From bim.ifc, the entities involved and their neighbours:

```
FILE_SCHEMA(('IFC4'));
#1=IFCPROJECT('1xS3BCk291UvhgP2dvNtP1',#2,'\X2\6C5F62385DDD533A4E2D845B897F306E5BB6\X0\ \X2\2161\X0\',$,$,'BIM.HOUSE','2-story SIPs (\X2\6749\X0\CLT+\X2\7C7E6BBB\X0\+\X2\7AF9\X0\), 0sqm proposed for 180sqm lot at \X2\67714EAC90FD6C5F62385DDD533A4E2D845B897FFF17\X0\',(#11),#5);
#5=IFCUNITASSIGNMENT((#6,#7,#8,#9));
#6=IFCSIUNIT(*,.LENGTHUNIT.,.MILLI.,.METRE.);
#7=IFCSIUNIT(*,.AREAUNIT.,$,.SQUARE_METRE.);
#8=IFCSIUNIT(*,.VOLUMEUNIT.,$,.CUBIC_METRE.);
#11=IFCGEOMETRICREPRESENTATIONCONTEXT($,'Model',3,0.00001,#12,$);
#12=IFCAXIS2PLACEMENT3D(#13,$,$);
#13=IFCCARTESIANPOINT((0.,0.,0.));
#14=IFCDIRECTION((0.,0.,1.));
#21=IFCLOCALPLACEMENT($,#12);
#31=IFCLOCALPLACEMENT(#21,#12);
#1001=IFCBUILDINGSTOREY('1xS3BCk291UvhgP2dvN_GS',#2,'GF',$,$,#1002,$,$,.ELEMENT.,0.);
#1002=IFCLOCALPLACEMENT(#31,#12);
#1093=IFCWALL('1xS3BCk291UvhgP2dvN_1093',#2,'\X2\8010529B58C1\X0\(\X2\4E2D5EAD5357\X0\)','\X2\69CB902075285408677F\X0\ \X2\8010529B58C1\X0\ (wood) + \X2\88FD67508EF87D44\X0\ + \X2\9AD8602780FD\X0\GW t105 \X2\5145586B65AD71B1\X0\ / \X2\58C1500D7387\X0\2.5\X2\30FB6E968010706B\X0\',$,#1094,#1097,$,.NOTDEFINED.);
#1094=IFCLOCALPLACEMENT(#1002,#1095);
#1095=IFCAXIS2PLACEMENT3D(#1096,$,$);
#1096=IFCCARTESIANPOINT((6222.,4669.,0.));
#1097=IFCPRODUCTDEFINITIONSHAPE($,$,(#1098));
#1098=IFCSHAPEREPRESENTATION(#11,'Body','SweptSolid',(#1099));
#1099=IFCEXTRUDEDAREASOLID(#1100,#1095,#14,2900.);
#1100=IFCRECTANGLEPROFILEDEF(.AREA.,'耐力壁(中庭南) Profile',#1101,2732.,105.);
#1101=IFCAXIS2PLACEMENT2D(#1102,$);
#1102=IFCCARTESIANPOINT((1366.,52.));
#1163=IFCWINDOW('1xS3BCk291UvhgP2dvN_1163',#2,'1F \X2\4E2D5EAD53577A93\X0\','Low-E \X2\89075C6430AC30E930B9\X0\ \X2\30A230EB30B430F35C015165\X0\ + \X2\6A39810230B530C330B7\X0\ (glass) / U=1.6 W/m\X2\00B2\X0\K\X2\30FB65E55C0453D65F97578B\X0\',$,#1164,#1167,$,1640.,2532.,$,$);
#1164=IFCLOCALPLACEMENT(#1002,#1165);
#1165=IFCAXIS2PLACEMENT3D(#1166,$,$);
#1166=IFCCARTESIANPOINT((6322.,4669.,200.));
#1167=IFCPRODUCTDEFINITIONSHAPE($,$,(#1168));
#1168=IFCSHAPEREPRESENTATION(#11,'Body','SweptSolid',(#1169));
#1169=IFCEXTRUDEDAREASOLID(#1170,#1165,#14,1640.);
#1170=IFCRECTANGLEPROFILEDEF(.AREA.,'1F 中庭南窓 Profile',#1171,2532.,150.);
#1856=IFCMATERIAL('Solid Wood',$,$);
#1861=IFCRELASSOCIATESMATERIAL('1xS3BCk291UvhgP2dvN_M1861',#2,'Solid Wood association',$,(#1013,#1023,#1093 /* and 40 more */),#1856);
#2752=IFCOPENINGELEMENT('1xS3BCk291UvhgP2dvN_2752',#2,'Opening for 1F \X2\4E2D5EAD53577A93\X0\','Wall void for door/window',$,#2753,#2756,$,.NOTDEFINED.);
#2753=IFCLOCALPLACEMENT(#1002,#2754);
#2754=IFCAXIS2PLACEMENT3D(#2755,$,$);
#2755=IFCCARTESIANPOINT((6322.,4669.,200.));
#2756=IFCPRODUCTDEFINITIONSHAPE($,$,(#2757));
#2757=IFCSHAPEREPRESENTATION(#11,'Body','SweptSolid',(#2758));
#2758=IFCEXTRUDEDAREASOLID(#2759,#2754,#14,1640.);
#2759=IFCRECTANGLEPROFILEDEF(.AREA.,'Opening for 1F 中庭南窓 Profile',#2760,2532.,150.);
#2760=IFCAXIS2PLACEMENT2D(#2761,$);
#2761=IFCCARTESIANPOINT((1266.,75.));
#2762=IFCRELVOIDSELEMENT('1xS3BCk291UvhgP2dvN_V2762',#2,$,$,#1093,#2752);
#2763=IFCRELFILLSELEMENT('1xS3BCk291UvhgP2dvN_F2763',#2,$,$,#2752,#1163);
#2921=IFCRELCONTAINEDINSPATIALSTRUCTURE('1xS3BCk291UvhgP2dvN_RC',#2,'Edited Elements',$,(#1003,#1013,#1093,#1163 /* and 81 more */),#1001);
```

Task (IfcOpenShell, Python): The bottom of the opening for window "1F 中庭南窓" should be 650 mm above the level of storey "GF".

```python
import numpy as np
import ifcopenshell
import ifcopenshell.api.geometry
import ifcopenshell.geom
import ifcopenshell.util.element
import ifcopenshell.util.placement
import ifcopenshell.util.shape
import ifcopenshell.util.unit

model = ifcopenshell.open("bim.ifc")
unit_scale = ifcopenshell.util.unit.calculate_unit_scale(model)

window = model.by_guid("1xS3BCk291UvhgP2dvN_1163")
opening = window.FillsVoids[0].RelatingOpeningElement
storey = ifcopenshell.util.element.get_container(window, ifc_class="IfcBuildingStorey")
level = ifcopenshell.util.placement.get_local_placement(storey.ObjectPlacement)[2, 3]

# The opening's origin need not be at the sill, so measure its lowest point.
shape = ifcopenshell.geom.create_shape(ifcopenshell.geom.settings(), opening)
bottom = ifcopenshell.util.shape.get_shape_bottom_elevation(shape, shape.geometry) / unit_scale
dz = level + 0.65 / unit_scale - bottom

shift = np.array([0.0, 0.0, dz])
# The window is not placed relative to its opening, so move both.
for product in (opening, window):
    matrix = ifcopenshell.util.placement.get_local_placement(product.ObjectPlacement)
    matrix[:3, 3] += shift
    ifcopenshell.api.geometry.edit_object_placement(model, product=product, matrix=matrix, is_si=False)

print(f"moved by {dz * unit_scale:+.3f} m")

model.write("bim_edited.ifc")
```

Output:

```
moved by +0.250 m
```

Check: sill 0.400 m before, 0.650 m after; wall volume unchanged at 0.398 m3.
